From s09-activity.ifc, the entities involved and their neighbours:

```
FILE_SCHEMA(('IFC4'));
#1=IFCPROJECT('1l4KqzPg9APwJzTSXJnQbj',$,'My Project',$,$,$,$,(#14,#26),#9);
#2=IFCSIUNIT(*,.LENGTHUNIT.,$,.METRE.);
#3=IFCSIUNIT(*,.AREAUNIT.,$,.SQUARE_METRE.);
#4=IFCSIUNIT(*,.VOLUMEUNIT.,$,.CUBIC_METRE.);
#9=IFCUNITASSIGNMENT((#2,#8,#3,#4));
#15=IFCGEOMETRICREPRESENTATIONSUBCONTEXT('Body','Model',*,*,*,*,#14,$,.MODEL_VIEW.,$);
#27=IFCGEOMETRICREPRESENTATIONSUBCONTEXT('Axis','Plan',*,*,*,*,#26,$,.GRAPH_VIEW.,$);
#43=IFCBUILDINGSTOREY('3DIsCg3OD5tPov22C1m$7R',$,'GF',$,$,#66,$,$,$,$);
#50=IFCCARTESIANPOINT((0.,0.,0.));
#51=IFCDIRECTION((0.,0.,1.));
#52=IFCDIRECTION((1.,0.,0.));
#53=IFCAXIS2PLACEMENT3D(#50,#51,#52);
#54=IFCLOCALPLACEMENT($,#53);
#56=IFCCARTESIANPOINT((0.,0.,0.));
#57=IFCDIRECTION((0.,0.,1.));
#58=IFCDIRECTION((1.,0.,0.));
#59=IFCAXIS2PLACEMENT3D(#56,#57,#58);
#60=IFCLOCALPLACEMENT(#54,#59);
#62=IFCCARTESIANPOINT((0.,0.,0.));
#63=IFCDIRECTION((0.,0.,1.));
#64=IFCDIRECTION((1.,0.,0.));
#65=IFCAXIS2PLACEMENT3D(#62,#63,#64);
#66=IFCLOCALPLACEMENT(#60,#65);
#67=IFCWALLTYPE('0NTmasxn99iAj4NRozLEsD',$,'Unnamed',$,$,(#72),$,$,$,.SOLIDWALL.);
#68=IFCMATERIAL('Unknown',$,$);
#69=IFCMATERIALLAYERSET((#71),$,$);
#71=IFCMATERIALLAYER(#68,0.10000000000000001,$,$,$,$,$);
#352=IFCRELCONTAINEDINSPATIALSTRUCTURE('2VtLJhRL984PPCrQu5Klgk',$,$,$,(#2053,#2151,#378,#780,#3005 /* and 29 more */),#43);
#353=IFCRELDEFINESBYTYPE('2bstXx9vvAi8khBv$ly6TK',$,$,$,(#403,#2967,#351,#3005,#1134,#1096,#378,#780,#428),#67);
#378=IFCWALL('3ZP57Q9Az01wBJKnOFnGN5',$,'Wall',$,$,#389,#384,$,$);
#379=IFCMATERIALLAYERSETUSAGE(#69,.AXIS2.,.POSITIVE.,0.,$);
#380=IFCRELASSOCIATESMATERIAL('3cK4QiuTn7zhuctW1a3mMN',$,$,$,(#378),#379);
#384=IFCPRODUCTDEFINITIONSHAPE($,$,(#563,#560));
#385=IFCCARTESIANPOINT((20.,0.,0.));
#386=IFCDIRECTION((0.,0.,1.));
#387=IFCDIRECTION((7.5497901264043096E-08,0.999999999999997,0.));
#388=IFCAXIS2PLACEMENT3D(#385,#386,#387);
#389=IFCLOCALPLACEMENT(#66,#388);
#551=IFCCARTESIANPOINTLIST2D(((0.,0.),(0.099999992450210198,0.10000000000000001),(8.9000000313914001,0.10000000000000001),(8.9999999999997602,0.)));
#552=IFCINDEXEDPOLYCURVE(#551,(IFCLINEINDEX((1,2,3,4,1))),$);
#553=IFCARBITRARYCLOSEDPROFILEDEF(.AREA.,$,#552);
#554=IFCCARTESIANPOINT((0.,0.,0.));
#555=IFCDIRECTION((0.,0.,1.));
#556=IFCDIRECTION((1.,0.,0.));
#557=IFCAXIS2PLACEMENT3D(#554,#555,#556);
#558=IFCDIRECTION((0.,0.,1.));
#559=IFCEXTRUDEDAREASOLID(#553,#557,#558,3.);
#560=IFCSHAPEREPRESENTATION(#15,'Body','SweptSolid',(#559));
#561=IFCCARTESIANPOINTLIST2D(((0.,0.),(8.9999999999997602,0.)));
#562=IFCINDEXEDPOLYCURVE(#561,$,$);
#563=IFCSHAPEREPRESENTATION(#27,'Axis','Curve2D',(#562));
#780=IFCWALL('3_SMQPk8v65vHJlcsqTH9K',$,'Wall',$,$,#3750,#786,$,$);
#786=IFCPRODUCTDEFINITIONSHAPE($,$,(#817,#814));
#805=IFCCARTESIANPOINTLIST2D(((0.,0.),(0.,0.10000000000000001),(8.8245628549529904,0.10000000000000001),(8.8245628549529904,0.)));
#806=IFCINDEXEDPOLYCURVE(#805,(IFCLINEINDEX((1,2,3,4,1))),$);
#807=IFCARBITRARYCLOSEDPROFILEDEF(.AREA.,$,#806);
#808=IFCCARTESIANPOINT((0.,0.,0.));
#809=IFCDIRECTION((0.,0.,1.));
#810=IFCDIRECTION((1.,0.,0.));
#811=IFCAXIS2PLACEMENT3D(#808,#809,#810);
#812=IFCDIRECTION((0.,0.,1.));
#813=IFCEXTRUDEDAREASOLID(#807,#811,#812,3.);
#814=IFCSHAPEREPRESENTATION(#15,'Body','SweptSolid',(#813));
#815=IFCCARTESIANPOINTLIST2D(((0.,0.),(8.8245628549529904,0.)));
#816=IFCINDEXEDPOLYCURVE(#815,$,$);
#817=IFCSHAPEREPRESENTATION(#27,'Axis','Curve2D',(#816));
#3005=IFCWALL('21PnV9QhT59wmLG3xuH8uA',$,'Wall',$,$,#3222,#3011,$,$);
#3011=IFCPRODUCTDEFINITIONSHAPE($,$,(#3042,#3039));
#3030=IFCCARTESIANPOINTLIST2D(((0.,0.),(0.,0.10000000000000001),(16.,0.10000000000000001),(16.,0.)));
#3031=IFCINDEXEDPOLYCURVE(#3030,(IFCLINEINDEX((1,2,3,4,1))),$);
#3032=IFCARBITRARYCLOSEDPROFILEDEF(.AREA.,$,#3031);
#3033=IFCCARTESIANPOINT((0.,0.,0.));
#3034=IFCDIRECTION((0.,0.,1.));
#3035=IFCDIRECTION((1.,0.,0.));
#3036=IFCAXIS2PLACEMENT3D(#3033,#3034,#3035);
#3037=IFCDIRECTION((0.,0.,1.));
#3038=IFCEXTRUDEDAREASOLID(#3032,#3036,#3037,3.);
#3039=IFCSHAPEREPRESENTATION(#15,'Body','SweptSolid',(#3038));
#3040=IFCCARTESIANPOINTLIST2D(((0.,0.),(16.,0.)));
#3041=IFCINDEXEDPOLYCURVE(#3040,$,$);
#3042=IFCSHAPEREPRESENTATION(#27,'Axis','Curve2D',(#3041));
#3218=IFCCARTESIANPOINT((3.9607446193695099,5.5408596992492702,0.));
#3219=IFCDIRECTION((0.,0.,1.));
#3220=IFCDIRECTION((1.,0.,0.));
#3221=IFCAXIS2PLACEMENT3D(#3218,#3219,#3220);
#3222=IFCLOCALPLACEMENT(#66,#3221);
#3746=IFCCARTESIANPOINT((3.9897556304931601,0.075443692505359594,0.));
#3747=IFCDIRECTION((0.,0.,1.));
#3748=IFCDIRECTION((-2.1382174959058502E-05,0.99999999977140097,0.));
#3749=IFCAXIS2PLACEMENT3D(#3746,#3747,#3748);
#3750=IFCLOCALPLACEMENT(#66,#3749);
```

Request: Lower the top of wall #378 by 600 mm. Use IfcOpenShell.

```python
import ifcopenshell
import ifcopenshell.geom
import ifcopenshell.util.representation
import ifcopenshell.util.shape
import ifcopenshell.util.unit

model = ifcopenshell.open("s09-activity.ifc")
unit_scale = ifcopenshell.util.unit.calculate_unit_scale(model)
settings = ifcopenshell.geom.settings()


def volume(element):
    """Net volume in cubic metres, openings subtracted."""
    shape = ifcopenshell.geom.create_shape(settings, element)
    return ifcopenshell.util.shape.get_volume(shape.geometry)


wall = model.by_id(378)
before = volume(wall)

body = ifcopenshell.util.representation.get_representation(wall, "Model", "Body")
solid = body.Items[0]
old_height = solid.Depth
solid.Depth -= 0.6 / unit_scale
after = volume(wall)

print(f"height {old_height:g} -> {solid.Depth:g}, volume {before:.3f} -> {after:.3f} m3")

model.write("s09-activity-out.ifc")
```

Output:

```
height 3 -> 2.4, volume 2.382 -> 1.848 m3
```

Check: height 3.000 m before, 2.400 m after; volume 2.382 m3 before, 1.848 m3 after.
